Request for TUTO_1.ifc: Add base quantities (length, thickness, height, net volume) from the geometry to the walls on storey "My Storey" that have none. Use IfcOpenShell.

First a look at what the model holds.

```python
import ifcopenshell
import ifcopenshell.util.element
import ifcopenshell.util.unit

model = ifcopenshell.open("TUTO_1.ifc")
print(model.schema)
for unit_type in ("LENGTHUNIT", "AREAUNIT", "VOLUMEUNIT"):
    print(unit_type, ifcopenshell.util.unit.calculate_unit_scale(model, unit_type))
storey = next(s for s in model.by_type("IfcBuildingStorey") if s.Name == "My Storey")
walls = [e for e in ifcopenshell.util.element.get_decomposition(storey) if e.is_a("IfcWall")]
for e in sorted(walls, key=lambda e: e.id()):
    print(e.id(), e.is_a(), e.Name, list(ifcopenshell.util.element.get_psets(e, qtos_only=True)), sep=" | ")
```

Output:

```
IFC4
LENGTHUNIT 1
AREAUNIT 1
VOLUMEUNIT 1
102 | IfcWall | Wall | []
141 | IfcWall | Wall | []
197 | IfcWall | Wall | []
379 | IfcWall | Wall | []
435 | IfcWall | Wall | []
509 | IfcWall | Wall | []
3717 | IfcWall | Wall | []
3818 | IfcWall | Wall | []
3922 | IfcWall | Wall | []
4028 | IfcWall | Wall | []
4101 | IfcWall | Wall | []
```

```python
import ifcopenshell
import ifcopenshell.api.pset
import ifcopenshell.geom
import ifcopenshell.util.element
import ifcopenshell.util.shape
import ifcopenshell.util.unit

model = ifcopenshell.open("TUTO_1.ifc")
unit_scale = ifcopenshell.util.unit.calculate_unit_scale(model)
volume_scale = ifcopenshell.util.unit.calculate_unit_scale(model, "VOLUMEUNIT")
settings = ifcopenshell.geom.settings()

storey = next(s for s in model.by_type("IfcBuildingStorey") if s.Name == "My Storey")
walls = [e for e in ifcopenshell.util.element.get_decomposition(storey) if e.is_a("IfcWall")]

for e in sorted(walls, key=lambda e: e.id()):
    if ifcopenshell.util.element.get_psets(e, qtos_only=True, should_inherit=False):
        continue
    # Geometry comes back in metres, in the element's own axes.
    shape = ifcopenshell.geom.create_shape(settings, e)
    values = {
        "Length": ifcopenshell.util.shape.get_x(shape.geometry) / unit_scale,
        "Width": ifcopenshell.util.shape.get_y(shape.geometry) / unit_scale,
        "Height": ifcopenshell.util.shape.get_z(shape.geometry) / unit_scale,
        "NetVolume": ifcopenshell.util.shape.get_volume(shape.geometry) / volume_scale,
    }
    qto = ifcopenshell.api.pset.add_qto(model, product=e, name="Qto_WallBaseQuantities")
    ifcopenshell.api.pset.edit_qto(model, qto=qto, properties=values)
    print(e.id(), {k: round(v, 3) for k, v in values.items()})

model.write("TUTO_1-out.ifc")
```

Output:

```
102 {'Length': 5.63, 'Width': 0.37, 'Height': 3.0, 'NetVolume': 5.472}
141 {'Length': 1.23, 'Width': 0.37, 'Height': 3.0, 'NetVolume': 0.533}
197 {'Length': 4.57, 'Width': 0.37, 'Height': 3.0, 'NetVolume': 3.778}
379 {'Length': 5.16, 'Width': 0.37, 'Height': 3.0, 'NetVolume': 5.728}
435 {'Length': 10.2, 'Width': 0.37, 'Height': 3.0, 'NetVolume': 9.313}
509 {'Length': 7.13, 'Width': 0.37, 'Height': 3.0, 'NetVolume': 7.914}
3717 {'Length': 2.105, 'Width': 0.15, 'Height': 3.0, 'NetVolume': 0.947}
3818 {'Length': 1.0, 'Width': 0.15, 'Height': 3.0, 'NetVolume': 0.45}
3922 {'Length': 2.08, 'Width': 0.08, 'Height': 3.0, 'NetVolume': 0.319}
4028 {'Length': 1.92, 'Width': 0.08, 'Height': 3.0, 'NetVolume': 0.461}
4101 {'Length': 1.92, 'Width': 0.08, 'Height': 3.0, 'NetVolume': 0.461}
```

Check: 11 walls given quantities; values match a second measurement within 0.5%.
